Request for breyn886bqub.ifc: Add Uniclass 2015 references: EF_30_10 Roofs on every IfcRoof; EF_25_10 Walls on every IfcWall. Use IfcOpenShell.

First a look at what the model holds.

```python
import ifcopenshell

model = ifcopenshell.open("breyn886bqub.ifc")
print(model.schema)
print("classifications:", [c.Name for c in model.by_type("IfcClassification")])
for ifc_class in ("IfcDoor", "IfcRoof", "IfcStair", "IfcWall", "IfcWindow"):
    print(ifc_class, len(model.by_type(ifc_class)))
```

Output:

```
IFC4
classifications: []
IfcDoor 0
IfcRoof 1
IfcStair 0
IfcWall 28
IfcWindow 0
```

```python
import ifcopenshell
import ifcopenshell.api.classification

model = ifcopenshell.open("breyn886bqub.ifc")

system = ifcopenshell.api.classification.add_classification(model, classification="Uniclass 2015")

codes = {
    "IfcRoof": ("EF_30_10", "Roofs"),
    "IfcWall": ("EF_25_10", "Walls"),
}
for ifc_class, (code, name) in codes.items():
    products = model.by_type(ifc_class)
    ifcopenshell.api.classification.add_reference(
        model, products=products, classification=system, identification=code, name=name
    )
    print(code, len(products))

model.write("breyn886bqub_edited.ifc")
```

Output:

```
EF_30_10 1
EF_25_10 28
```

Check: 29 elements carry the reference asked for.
